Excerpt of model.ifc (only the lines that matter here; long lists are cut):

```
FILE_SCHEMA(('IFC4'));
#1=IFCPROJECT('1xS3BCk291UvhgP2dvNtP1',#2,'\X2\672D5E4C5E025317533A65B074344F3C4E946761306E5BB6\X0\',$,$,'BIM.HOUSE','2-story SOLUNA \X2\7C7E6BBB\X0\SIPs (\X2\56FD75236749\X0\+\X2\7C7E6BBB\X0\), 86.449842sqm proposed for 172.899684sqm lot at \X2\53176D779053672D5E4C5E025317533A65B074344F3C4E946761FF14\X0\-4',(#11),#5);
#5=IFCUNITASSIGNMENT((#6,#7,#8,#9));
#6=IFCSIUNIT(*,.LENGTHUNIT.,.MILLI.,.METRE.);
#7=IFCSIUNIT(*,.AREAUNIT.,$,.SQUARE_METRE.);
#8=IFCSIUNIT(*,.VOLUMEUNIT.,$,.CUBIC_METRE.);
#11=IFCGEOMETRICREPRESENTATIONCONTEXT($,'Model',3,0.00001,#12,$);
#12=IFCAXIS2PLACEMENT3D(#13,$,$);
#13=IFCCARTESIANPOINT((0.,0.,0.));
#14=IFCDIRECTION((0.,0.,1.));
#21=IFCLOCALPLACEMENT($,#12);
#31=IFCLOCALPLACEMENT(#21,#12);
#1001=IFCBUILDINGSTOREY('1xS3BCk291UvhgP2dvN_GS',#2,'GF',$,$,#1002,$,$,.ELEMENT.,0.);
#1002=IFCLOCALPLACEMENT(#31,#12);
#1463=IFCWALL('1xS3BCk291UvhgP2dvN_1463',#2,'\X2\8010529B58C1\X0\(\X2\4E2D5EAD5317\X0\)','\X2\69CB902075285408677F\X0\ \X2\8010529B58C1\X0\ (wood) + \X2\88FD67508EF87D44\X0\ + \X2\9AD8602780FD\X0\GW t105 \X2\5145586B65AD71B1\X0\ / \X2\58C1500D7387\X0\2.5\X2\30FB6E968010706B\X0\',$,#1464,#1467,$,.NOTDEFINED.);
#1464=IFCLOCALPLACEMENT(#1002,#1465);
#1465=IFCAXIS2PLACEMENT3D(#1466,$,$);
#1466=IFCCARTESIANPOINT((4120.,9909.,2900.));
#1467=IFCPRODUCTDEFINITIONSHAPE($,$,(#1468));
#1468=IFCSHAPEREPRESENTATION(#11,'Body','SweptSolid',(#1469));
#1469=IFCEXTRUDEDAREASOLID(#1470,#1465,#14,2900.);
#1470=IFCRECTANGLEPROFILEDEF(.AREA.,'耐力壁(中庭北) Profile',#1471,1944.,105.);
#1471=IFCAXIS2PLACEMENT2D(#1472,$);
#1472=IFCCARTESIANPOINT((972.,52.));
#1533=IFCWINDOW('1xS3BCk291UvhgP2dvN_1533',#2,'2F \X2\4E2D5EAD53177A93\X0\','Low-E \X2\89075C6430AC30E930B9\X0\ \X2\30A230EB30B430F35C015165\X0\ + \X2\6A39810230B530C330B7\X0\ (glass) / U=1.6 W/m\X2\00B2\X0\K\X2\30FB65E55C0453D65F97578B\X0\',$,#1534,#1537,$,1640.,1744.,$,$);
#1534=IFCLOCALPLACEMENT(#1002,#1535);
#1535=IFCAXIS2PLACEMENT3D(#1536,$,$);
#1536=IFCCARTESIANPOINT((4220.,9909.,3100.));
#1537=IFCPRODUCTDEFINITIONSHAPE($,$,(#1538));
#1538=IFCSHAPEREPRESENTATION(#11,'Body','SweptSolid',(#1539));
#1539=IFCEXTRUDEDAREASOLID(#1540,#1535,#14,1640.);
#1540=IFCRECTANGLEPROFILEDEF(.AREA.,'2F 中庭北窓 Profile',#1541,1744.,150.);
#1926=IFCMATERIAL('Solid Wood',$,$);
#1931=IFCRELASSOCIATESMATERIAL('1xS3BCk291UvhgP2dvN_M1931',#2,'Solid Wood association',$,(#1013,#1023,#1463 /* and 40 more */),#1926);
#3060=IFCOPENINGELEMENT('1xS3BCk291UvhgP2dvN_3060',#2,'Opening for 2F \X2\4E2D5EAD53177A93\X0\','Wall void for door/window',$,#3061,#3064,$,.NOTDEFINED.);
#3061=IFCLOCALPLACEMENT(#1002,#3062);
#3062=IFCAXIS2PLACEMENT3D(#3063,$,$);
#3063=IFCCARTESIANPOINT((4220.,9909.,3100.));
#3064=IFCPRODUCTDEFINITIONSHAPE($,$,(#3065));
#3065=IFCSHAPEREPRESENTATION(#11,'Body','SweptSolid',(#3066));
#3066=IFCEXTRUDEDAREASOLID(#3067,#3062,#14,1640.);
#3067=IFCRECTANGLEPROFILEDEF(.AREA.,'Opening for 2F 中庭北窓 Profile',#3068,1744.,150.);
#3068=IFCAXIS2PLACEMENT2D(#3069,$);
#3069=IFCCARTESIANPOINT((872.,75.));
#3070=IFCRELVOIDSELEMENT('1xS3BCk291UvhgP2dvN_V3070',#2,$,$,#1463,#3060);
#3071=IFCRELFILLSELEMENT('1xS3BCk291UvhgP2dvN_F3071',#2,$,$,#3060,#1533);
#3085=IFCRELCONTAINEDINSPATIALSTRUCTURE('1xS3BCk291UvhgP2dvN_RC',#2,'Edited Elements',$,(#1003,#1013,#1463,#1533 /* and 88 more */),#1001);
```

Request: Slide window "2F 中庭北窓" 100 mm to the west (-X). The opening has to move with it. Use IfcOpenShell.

```python
import ifcopenshell
import ifcopenshell.api.geometry
import ifcopenshell.util.placement

model = ifcopenshell.open("model.ifc")

window = model.by_guid("1xS3BCk291UvhgP2dvN_1533")
opening = window.FillsVoids[0].RelatingOpeningElement
wall = opening.VoidsElements[0].RelatingBuildingElement

wall_matrix = ifcopenshell.util.placement.get_local_placement(wall.ObjectPlacement)
shift = wall_matrix[:3, 0] * -100.0
before = ifcopenshell.util.placement.get_local_placement(window.ObjectPlacement)[:3, 3].copy()

# The window is not placed relative to its opening, so move both.
for product in (opening, window):
    matrix = ifcopenshell.util.placement.get_local_placement(product.ObjectPlacement)
    matrix[:3, 3] += shift
    ifcopenshell.api.geometry.edit_object_placement(model, product=product, matrix=matrix, is_si=False)

after = ifcopenshell.util.placement.get_local_placement(window.ObjectPlacement)[:3, 3]
print("window moved by", (after - before).round(3) + 0.0)

model.write("model_updated.ifc")
```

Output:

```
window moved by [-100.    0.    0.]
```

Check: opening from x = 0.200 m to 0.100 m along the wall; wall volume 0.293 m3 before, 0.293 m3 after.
